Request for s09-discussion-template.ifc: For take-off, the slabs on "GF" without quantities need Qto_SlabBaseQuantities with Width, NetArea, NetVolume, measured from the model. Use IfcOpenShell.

First a look at what the model holds.

```python
import ifcopenshell
import ifcopenshell.util.element
import ifcopenshell.util.unit

model = ifcopenshell.open("s09-discussion-template.ifc")
print(model.schema)
for unit_type in ("LENGTHUNIT", "AREAUNIT", "VOLUMEUNIT"):
    print(unit_type, ifcopenshell.util.unit.calculate_unit_scale(model, unit_type))
storey = next(s for s in model.by_type("IfcBuildingStorey") if s.Name == "GF")
slabs = [e for e in ifcopenshell.util.element.get_decomposition(storey) if e.is_a("IfcSlab")]
for e in sorted(slabs, key=lambda e: e.id()):
    print(e.id(), e.is_a(), e.Name, list(ifcopenshell.util.element.get_psets(e, qtos_only=True)), sep=" | ")
```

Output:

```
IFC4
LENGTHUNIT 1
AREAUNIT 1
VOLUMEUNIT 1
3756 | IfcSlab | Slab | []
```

```python
import ifcopenshell
import ifcopenshell.api.pset
import ifcopenshell.geom
import ifcopenshell.util.element
import ifcopenshell.util.shape
import ifcopenshell.util.unit

model = ifcopenshell.open("s09-discussion-template.ifc")
unit_scale = ifcopenshell.util.unit.calculate_unit_scale(model)
area_scale = ifcopenshell.util.unit.calculate_unit_scale(model, "AREAUNIT")
volume_scale = ifcopenshell.util.unit.calculate_unit_scale(model, "VOLUMEUNIT")
settings = ifcopenshell.geom.settings()

storey = next(s for s in model.by_type("IfcBuildingStorey") if s.Name == "GF")
slabs = [e for e in ifcopenshell.util.element.get_decomposition(storey) if e.is_a("IfcSlab")]

for e in sorted(slabs, key=lambda e: e.id()):
    if ifcopenshell.util.element.get_psets(e, qtos_only=True, should_inherit=False):
        continue
    # Geometry comes back in metres, in the element's own axes.
    shape = ifcopenshell.geom.create_shape(settings, e)
    values = {
        "Width": ifcopenshell.util.shape.get_z(shape.geometry) / unit_scale,
        "NetArea": ifcopenshell.util.shape.get_footprint_area(shape.geometry) / area_scale,
        "NetVolume": ifcopenshell.util.shape.get_volume(shape.geometry) / volume_scale,
    }
    qto = ifcopenshell.api.pset.add_qto(model, product=e, name="Qto_SlabBaseQuantities")
    ifcopenshell.api.pset.edit_qto(model, qto=qto, properties=values)
    print(e.id(), {k: round(v, 3) for k, v in values.items()})

model.write("s09-discussion-template_edited.ifc")
```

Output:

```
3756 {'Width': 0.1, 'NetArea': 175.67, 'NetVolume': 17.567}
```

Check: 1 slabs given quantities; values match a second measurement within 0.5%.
